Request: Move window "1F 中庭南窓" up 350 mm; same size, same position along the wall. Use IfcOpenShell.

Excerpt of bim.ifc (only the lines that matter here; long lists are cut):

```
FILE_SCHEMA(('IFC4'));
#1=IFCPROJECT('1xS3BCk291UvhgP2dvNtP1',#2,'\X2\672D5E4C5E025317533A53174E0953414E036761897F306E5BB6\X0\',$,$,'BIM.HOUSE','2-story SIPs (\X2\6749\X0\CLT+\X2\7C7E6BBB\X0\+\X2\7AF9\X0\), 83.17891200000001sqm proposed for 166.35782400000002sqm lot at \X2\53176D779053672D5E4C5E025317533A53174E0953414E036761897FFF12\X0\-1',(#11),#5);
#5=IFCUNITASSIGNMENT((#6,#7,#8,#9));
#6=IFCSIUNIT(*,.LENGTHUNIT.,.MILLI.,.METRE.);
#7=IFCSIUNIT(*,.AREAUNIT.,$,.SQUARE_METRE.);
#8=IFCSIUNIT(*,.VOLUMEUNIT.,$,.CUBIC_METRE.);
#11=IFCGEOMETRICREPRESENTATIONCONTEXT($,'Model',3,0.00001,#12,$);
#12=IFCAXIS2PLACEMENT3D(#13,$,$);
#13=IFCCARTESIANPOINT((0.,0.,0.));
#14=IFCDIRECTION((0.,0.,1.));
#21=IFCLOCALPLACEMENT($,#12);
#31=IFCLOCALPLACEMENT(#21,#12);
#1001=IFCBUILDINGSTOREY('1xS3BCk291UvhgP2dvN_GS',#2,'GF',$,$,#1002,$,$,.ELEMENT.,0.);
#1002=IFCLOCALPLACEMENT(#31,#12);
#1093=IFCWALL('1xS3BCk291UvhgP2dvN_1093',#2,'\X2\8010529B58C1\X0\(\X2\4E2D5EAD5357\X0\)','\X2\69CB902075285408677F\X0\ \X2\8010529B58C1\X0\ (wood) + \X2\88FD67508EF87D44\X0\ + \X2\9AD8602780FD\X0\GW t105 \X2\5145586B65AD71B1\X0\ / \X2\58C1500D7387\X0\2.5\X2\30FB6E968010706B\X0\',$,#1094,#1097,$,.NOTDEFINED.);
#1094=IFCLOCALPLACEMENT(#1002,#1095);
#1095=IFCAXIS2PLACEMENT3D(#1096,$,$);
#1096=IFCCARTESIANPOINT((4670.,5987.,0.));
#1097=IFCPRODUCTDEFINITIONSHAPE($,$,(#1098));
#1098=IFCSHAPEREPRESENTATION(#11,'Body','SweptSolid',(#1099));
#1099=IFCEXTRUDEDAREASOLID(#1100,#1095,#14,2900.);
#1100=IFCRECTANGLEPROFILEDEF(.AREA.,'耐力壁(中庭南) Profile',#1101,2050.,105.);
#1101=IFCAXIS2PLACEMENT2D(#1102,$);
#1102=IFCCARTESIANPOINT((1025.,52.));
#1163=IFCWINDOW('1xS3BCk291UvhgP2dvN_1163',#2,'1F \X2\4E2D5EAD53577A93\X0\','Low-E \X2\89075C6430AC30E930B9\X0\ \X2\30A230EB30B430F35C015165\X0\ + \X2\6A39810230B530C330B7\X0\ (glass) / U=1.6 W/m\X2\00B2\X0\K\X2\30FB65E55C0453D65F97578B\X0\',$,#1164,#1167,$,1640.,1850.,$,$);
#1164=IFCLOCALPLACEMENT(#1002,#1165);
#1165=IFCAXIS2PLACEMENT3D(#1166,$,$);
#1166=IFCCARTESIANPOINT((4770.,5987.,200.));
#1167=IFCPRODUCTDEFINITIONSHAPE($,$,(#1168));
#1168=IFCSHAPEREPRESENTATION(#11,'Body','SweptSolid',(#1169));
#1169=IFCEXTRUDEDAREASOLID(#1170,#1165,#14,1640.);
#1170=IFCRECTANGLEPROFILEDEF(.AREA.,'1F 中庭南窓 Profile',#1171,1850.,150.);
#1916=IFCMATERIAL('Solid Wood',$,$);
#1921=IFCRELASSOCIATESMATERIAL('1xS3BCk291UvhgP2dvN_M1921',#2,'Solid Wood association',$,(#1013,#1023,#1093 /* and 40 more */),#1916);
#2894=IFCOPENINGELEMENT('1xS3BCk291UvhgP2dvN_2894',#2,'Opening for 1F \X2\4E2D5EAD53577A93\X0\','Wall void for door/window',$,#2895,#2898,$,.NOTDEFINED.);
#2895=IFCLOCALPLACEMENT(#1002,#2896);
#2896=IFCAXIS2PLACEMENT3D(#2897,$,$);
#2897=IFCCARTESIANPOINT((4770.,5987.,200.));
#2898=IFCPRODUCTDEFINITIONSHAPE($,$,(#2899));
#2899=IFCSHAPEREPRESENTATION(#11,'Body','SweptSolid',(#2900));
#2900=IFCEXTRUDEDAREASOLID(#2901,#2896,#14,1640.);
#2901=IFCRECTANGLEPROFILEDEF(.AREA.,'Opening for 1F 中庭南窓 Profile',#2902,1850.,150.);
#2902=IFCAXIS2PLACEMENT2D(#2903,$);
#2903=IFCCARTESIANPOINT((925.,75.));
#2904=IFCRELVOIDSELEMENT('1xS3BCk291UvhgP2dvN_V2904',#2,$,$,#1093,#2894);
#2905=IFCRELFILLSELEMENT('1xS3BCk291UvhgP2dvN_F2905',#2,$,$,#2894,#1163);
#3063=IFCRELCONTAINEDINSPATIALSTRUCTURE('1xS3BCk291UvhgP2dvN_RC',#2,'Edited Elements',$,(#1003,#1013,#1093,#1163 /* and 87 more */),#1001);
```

```python
import numpy as np
import ifcopenshell
import ifcopenshell.api.geometry
import ifcopenshell.util.placement
import ifcopenshell.util.unit

model = ifcopenshell.open("bim.ifc")
unit_scale = ifcopenshell.util.unit.calculate_unit_scale(model)

window = model.by_id(1163)
opening = window.FillsVoids[0].RelatingOpeningElement
dz = 0.35 / unit_scale

shift = np.array([0.0, 0.0, dz])
# The window is not placed relative to its opening, so move both.
for product in (opening, window):
    matrix = ifcopenshell.util.placement.get_local_placement(product.ObjectPlacement)
    matrix[:3, 3] += shift
    ifcopenshell.api.geometry.edit_object_placement(model, product=product, matrix=matrix, is_si=False)

print(f"moved by {dz * unit_scale:+.3f} m")

model.write("bim-out.ifc")
```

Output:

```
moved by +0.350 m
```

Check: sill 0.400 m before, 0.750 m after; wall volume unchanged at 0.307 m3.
